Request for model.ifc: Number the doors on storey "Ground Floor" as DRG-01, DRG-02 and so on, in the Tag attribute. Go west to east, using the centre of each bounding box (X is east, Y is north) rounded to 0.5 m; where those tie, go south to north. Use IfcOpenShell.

First a look at what the model holds.

```python
import ifcopenshell
import ifcopenshell.util.element
import ifcopenshell.util.placement

model = ifcopenshell.open("model.ifc")
print(model.schema)
storey = next(s for s in model.by_type("IfcBuildingStorey") if s.Name == "Ground Floor")
doors = [e for e in ifcopenshell.util.element.get_decomposition(storey) if e.is_a("IfcDoor")]
for e in sorted(doors, key=lambda e: e.id()):
    origin = ifcopenshell.util.placement.get_local_placement(e.ObjectPlacement)[:3, 3]
    print(e.id(), e.Tag, e.Name, origin.round(2) + 0.0, sep=" | ")
```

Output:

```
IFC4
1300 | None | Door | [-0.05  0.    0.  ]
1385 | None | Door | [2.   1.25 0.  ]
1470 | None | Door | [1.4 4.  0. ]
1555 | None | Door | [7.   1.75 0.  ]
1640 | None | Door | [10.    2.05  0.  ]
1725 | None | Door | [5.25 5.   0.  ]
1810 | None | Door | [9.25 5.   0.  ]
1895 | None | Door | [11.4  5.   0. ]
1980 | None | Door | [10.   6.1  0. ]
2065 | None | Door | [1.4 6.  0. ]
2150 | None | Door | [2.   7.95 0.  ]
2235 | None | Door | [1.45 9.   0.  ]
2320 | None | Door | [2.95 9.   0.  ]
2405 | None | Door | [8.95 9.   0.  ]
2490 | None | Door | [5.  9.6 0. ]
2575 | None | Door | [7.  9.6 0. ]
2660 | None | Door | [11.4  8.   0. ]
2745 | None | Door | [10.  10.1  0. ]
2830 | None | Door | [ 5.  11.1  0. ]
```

```python
import ifcopenshell
import ifcopenshell.geom
import ifcopenshell.util.element
import ifcopenshell.util.shape

model = ifcopenshell.open("model.ifc")
settings = ifcopenshell.geom.settings()
settings.set("use-world-coords", True)


def centre(element):
    shape = ifcopenshell.geom.create_shape(settings, element)
    return ifcopenshell.util.shape.get_bbox_centroid(shape.geometry)


storey = next(s for s in model.by_type("IfcBuildingStorey") if s.Name == "Ground Floor")
doors = [e for e in ifcopenshell.util.element.get_decomposition(storey) if e.is_a("IfcDoor")]

# Insertion points can sit at a corner or the storey origin, so sort by the geometry (in metres).
centres = {e: centre(e) for e in doors}
doors.sort(key=lambda e: (round(centres[e][0] / 0.5), centres[e][1]))

for i, e in enumerate(doors, start=1):
    number = f"DRG-{i:02d}"
    e.Tag = number
    print(e.id(), number)

model.write("model_updated.ifc")
```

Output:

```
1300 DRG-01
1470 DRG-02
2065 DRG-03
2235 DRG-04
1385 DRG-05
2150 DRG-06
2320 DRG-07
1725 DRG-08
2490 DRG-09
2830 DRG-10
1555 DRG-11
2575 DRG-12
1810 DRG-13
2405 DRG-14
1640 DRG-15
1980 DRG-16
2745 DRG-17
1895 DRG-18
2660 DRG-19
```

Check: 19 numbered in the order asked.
